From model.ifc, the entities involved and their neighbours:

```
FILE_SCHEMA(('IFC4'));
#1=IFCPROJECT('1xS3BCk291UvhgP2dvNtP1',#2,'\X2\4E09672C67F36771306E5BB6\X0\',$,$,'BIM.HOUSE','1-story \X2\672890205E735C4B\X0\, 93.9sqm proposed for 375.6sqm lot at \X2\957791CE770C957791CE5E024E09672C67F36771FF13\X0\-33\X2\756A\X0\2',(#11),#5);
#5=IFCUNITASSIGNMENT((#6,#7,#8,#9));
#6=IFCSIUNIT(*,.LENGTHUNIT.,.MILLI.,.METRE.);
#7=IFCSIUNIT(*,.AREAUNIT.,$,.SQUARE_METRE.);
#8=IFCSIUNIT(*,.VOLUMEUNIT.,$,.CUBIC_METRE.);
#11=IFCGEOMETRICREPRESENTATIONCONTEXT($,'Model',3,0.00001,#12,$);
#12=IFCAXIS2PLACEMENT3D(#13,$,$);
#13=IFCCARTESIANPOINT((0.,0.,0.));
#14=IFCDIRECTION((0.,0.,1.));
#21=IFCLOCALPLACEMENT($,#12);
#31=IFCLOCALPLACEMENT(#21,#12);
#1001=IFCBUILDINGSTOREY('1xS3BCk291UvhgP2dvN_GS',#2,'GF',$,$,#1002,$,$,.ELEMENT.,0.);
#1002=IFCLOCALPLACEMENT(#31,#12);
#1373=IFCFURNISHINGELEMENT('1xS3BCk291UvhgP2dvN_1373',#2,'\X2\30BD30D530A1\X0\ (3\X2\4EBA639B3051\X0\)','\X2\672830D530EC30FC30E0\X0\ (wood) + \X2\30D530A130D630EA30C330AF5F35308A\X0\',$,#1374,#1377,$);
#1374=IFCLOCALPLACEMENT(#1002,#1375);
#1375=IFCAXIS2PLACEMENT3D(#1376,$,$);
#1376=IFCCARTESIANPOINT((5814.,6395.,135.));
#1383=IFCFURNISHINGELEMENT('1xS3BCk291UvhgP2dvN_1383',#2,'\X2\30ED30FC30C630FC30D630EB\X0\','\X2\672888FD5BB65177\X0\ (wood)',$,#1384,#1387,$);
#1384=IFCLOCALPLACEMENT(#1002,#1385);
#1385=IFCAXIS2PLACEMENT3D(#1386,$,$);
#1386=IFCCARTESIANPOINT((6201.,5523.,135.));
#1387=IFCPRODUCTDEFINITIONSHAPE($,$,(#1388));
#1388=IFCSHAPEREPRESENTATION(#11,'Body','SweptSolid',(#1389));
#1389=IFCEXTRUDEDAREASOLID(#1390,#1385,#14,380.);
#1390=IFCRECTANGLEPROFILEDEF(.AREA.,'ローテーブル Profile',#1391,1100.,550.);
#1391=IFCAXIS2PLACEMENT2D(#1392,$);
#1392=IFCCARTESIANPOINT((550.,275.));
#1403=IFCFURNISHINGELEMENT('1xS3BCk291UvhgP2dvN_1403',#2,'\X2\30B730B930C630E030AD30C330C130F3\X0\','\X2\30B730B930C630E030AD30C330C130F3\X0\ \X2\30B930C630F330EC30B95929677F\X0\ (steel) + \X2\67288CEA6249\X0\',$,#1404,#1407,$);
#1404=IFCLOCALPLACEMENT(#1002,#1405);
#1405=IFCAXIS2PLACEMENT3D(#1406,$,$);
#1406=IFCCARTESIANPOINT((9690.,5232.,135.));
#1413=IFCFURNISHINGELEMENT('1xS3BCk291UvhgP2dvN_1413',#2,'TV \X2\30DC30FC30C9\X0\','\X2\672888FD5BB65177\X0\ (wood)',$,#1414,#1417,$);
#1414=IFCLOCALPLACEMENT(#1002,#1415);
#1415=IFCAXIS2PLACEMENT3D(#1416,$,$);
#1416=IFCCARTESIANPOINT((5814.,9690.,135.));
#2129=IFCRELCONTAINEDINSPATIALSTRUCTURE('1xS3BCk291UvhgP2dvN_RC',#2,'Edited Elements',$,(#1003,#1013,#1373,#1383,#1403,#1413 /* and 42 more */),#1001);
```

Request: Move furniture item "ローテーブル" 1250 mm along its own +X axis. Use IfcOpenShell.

```python
import ifcopenshell
import ifcopenshell.api.geometry
import ifcopenshell.util.placement
import ifcopenshell.util.unit

model = ifcopenshell.open("model.ifc")
unit_scale = ifcopenshell.util.unit.calculate_unit_scale(model)

item = model.by_guid("1xS3BCk291UvhgP2dvN_1383")
matrix = ifcopenshell.util.placement.get_local_placement(item.ObjectPlacement)
matrix[:3, 3] += matrix[:3, 0] * 1.25 / unit_scale
ifcopenshell.api.geometry.edit_object_placement(model, product=item, matrix=matrix, is_si=False)

print(ifcopenshell.util.placement.get_local_placement(item.ObjectPlacement).round(3) + 0.0)

model.write("model_updated.ifc")
```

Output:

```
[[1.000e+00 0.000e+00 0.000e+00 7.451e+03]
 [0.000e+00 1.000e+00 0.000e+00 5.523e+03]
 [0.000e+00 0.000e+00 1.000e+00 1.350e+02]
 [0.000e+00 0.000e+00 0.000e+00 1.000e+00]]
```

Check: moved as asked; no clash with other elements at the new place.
